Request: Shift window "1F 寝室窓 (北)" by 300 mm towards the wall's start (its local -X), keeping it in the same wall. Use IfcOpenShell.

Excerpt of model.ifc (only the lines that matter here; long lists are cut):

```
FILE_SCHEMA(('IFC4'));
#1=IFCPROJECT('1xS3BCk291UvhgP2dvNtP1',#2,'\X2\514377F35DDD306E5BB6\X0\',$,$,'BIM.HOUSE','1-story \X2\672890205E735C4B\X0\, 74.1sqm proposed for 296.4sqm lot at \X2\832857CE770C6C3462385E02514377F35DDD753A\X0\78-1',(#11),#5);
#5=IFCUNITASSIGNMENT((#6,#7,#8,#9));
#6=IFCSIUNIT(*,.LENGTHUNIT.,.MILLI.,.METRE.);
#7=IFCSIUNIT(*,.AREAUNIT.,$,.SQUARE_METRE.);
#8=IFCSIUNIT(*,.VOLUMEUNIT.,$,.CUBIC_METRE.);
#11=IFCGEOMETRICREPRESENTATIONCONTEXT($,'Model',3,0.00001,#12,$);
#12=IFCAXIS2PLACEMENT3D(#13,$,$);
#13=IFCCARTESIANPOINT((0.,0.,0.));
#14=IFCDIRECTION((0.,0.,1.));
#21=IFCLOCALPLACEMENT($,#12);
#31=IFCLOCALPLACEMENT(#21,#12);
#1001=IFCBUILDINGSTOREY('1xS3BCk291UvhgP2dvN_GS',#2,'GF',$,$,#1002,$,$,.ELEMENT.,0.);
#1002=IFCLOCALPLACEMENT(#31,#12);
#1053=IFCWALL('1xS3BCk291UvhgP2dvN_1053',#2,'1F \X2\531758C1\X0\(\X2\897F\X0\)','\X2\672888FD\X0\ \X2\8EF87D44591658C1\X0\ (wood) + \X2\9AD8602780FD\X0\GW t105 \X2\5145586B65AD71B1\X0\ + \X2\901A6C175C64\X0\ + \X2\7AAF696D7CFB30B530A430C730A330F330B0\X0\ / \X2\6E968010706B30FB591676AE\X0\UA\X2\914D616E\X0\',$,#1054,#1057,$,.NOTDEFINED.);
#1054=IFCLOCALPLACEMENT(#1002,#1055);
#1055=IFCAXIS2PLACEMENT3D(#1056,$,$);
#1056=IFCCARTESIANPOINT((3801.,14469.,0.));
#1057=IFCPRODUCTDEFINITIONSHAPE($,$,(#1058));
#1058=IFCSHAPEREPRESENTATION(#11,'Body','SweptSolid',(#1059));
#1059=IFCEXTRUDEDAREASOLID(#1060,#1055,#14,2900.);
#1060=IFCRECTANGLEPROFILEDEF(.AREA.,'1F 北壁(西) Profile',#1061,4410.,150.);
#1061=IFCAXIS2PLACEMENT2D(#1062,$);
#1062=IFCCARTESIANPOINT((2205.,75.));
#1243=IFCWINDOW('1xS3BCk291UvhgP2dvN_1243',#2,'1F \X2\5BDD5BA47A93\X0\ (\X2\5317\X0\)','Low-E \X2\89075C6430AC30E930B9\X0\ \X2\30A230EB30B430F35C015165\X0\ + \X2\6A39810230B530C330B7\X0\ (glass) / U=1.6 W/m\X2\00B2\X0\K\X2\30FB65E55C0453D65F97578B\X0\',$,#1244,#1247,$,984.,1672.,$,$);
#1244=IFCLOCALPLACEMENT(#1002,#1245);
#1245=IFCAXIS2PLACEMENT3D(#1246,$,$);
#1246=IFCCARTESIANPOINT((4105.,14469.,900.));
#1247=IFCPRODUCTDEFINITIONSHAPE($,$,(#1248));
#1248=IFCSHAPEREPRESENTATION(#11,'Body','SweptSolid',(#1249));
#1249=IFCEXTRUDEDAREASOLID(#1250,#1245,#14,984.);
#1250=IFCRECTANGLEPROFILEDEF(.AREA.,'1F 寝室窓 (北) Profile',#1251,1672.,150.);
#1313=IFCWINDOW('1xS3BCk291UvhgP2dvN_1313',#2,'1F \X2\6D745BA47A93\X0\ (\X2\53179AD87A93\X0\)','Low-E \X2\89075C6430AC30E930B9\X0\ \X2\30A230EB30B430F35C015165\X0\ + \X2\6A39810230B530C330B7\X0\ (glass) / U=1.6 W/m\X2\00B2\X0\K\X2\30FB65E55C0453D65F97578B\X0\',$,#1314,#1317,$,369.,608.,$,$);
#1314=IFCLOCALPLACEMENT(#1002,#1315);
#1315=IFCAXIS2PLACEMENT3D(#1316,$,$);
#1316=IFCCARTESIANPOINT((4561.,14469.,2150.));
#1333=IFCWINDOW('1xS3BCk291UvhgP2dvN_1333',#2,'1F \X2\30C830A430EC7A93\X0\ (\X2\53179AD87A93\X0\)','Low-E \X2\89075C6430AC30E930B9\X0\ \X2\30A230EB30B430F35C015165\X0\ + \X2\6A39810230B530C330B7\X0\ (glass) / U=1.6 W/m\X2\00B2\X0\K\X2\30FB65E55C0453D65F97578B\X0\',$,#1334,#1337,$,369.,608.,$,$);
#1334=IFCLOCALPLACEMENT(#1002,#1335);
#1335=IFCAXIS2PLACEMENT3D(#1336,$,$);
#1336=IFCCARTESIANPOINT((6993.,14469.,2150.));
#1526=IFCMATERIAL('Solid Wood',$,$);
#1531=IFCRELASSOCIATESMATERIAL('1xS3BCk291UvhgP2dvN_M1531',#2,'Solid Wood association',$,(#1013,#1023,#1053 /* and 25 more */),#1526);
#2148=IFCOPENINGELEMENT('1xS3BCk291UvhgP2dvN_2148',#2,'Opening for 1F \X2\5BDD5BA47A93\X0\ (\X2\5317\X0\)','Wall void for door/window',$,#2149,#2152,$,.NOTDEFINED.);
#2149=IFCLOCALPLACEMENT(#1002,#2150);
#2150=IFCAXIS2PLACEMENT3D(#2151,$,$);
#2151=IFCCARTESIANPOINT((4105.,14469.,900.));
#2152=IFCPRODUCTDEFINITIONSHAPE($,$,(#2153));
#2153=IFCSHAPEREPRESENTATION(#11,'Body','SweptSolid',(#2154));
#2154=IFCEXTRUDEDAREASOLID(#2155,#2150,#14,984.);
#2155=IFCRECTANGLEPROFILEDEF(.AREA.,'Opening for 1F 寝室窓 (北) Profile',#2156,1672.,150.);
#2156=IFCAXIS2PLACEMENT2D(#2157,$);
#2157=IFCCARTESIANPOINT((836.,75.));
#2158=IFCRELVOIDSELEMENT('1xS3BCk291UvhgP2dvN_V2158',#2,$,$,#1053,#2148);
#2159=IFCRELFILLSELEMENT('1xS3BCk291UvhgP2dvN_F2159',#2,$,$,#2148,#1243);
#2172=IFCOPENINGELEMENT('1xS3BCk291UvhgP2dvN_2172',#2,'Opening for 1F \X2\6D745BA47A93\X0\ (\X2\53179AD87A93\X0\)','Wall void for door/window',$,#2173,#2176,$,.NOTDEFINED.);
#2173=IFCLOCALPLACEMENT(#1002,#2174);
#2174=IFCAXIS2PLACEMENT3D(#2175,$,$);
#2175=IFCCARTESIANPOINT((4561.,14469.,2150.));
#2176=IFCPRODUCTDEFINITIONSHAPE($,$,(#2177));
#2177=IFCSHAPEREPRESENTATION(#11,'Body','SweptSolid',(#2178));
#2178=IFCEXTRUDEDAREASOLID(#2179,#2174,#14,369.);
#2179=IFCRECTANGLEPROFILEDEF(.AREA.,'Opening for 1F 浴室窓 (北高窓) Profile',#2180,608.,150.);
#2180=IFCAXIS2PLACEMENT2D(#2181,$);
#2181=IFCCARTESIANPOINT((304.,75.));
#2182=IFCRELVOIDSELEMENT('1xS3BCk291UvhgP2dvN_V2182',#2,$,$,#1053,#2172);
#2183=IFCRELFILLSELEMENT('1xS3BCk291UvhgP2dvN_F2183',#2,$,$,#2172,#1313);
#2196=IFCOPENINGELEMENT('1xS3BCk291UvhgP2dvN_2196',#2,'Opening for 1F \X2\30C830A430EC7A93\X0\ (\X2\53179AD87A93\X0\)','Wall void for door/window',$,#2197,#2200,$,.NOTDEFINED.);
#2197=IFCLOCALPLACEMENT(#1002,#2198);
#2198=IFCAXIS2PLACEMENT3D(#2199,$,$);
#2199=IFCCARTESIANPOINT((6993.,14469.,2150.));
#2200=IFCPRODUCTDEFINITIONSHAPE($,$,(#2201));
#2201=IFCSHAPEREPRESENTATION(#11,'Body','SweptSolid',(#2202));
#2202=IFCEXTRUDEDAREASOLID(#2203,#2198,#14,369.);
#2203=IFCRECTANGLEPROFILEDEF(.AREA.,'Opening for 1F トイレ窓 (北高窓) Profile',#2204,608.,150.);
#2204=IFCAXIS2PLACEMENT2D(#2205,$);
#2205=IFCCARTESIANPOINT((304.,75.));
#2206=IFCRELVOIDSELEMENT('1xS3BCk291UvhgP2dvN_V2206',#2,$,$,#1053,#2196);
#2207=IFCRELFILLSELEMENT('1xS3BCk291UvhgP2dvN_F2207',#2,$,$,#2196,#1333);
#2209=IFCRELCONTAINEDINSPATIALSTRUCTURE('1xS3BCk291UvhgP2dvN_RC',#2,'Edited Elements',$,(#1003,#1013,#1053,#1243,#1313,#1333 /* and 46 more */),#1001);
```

```python
import ifcopenshell
import ifcopenshell.api.geometry
import ifcopenshell.util.placement

model = ifcopenshell.open("model.ifc")

window = model.by_guid("1xS3BCk291UvhgP2dvN_1243")
opening = window.FillsVoids[0].RelatingOpeningElement
wall = opening.VoidsElements[0].RelatingBuildingElement

wall_matrix = ifcopenshell.util.placement.get_local_placement(wall.ObjectPlacement)
shift = wall_matrix[:3, 0] * -300.0
before = ifcopenshell.util.placement.get_local_placement(window.ObjectPlacement)[:3, 3].copy()

# The window is not placed relative to its opening, so move both.
for product in (opening, window):
    matrix = ifcopenshell.util.placement.get_local_placement(product.ObjectPlacement)
    matrix[:3, 3] += shift
    ifcopenshell.api.geometry.edit_object_placement(model, product=product, matrix=matrix, is_si=False)

after = ifcopenshell.util.placement.get_local_placement(window.ObjectPlacement)[:3, 3]
print("window moved by", (after - before).round(3) + 0.0)

model.write("model_updated.ifc")
```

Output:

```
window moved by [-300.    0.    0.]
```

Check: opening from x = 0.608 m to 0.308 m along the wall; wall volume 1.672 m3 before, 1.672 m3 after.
